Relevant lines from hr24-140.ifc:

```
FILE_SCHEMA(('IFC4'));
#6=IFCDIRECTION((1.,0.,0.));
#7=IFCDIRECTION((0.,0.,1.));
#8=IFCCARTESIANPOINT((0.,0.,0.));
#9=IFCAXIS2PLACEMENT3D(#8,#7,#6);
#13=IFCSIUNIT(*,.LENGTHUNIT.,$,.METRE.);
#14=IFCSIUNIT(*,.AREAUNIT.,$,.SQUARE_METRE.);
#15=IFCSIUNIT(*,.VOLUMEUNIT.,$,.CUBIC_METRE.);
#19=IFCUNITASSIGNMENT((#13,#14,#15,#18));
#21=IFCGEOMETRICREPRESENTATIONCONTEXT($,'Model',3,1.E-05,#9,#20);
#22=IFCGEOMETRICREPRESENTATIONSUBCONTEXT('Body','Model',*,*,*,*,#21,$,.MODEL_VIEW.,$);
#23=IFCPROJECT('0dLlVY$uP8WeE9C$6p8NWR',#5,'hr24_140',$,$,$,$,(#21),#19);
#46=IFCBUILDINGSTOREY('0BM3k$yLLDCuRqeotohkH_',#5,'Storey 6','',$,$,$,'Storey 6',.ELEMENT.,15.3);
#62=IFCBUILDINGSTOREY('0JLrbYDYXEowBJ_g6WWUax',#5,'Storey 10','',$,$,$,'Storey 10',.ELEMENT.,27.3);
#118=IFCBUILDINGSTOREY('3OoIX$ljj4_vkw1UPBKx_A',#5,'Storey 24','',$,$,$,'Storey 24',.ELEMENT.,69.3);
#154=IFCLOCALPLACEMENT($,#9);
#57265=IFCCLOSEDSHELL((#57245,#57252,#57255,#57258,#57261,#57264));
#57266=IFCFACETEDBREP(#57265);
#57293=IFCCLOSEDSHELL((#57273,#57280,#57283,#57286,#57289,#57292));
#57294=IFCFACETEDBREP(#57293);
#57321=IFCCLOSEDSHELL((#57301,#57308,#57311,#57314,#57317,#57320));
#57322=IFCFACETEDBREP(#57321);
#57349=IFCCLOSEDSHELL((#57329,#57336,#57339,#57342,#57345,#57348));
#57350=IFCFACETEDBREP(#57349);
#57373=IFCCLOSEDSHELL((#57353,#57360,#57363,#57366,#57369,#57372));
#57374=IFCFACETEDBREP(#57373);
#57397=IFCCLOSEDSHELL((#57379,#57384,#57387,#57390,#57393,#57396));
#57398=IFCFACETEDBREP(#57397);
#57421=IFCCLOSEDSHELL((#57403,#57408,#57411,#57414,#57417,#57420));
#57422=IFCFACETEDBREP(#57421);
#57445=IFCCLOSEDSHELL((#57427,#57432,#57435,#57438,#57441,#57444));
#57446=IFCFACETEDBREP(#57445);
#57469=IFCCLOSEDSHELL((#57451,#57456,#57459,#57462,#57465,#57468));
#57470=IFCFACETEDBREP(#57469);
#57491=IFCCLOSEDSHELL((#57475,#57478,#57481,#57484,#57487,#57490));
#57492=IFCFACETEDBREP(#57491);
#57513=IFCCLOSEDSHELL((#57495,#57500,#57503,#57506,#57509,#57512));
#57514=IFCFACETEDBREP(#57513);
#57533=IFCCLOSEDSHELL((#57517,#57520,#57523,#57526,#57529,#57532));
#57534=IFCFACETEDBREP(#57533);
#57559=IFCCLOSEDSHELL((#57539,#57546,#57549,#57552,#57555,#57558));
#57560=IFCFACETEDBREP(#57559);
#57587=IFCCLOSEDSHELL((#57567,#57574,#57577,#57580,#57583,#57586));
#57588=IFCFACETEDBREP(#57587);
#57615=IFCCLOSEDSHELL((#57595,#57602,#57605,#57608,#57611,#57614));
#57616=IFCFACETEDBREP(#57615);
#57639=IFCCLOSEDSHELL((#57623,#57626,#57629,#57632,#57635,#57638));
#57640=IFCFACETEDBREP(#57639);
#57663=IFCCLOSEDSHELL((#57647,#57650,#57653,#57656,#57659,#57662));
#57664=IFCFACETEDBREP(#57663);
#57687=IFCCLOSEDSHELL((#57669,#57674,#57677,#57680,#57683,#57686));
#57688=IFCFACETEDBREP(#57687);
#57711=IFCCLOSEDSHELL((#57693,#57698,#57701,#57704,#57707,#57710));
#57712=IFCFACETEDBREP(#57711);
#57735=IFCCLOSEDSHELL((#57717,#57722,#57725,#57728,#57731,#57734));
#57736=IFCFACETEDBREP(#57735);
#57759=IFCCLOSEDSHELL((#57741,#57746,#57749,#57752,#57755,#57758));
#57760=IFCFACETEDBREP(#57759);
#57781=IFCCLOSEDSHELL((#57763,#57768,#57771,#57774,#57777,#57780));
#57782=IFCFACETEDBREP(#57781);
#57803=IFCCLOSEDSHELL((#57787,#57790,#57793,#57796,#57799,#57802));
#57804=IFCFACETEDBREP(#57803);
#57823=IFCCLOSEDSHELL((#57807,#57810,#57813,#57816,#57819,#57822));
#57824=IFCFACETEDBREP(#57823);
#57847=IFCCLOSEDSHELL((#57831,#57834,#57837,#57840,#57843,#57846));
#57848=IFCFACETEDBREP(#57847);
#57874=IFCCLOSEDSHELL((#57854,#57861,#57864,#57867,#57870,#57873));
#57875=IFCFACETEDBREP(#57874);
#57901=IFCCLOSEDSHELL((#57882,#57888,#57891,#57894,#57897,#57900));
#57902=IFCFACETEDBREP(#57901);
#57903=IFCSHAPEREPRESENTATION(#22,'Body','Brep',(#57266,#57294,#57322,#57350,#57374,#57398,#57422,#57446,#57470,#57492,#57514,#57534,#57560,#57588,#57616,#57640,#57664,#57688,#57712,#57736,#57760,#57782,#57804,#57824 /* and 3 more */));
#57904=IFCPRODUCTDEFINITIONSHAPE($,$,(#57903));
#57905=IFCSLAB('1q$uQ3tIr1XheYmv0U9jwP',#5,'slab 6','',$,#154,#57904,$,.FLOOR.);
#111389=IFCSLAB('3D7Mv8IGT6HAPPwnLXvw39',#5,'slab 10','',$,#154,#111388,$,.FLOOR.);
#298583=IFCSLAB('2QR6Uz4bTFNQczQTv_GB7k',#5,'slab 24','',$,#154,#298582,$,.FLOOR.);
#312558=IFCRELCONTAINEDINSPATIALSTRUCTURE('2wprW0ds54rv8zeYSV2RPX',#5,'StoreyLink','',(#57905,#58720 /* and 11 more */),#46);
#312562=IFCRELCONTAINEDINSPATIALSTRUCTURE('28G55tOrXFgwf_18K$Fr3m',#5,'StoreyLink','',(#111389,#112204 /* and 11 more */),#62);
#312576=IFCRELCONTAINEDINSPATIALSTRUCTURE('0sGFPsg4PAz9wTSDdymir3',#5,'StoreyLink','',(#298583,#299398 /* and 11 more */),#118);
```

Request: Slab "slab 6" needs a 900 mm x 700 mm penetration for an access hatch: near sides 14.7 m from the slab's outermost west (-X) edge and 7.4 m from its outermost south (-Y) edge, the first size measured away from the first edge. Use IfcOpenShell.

```python
import numpy as np
import ifcopenshell
import ifcopenshell.api.feature
import ifcopenshell.api.geometry
import ifcopenshell.api.root
import ifcopenshell.geom
import ifcopenshell.util.placement
import ifcopenshell.util.representation
import ifcopenshell.util.shape
import ifcopenshell.util.unit

model = ifcopenshell.open("hr24-140.ifc")
unit_scale = ifcopenshell.util.unit.calculate_unit_scale(model)
settings = ifcopenshell.geom.settings()


def volume(element):
    """Net volume in cubic metres, openings subtracted."""
    shape = ifcopenshell.geom.create_shape(settings, element)
    return ifcopenshell.util.shape.get_volume(shape.geometry)


slab = model.by_guid("1q$uQ3tIr1XheYmv0U9jwP")
before = volume(slab)

# Extent in the slab's own axes, in metres. The edges named are its -X and -Y sides.
slab_shape = ifcopenshell.geom.create_shape(settings, slab)
vertices = ifcopenshell.util.shape.get_vertices(slab_shape.geometry)
x_min, y_min, bottom = vertices.min(axis=0)
top = vertices[:, 2].max()

opening = ifcopenshell.api.root.create_entity(model, ifc_class="IfcOpeningElement", name="Access hatch opening", predefined_type="OPENING")
context = ifcopenshell.util.representation.get_context(model, "Model", "Body", "MODEL_VIEW")
width, depth = 0.9, 0.7
outline = [(0.0, 0.0), (width, 0.0), (width, depth), (0.0, depth), (0.0, 0.0)]
# Overshoot both faces by 50 mm so the cut is clean.
shape = ifcopenshell.api.geometry.add_slab_representation(
    model, context=context, depth=top - bottom + 0.1, polyline=outline
)
ifcopenshell.api.geometry.assign_representation(model, product=opening, representation=shape)

matrix = ifcopenshell.util.placement.get_local_placement(slab.ObjectPlacement)
matrix[:, 3] = matrix @ np.append(np.array([x_min + 14.7, y_min + 7.4, bottom - 0.05]) / unit_scale, 1.0)
ifcopenshell.api.geometry.edit_object_placement(model, product=opening, matrix=matrix, is_si=False)
ifcopenshell.api.feature.add_feature(model, feature=opening, element=slab)

after = volume(slab)

print(f"slab volume {before:.3f} -> {after:.3f} m3")

model.write("hr24-140_v2.ifc")
```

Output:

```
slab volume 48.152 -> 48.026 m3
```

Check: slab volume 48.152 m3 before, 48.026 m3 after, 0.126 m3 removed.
